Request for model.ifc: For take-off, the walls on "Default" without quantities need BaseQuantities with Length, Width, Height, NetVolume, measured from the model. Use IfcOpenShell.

First a look at what the model holds.

```python
import ifcopenshell
import ifcopenshell.util.element
import ifcopenshell.util.unit

model = ifcopenshell.open("model.ifc")
print(model.schema)
for unit_type in ("LENGTHUNIT", "AREAUNIT", "VOLUMEUNIT"):
    print(unit_type, ifcopenshell.util.unit.calculate_unit_scale(model, unit_type))
storey = next(s for s in model.by_type("IfcBuildingStorey") if s.Name == "Default")
walls = [e for e in ifcopenshell.util.element.get_decomposition(storey) if e.is_a("IfcWall")]
for e in sorted(walls, key=lambda e: e.id()):
    print(e.id(), e.is_a(), e.Name, list(ifcopenshell.util.element.get_psets(e, qtos_only=True)), sep=" | ")
```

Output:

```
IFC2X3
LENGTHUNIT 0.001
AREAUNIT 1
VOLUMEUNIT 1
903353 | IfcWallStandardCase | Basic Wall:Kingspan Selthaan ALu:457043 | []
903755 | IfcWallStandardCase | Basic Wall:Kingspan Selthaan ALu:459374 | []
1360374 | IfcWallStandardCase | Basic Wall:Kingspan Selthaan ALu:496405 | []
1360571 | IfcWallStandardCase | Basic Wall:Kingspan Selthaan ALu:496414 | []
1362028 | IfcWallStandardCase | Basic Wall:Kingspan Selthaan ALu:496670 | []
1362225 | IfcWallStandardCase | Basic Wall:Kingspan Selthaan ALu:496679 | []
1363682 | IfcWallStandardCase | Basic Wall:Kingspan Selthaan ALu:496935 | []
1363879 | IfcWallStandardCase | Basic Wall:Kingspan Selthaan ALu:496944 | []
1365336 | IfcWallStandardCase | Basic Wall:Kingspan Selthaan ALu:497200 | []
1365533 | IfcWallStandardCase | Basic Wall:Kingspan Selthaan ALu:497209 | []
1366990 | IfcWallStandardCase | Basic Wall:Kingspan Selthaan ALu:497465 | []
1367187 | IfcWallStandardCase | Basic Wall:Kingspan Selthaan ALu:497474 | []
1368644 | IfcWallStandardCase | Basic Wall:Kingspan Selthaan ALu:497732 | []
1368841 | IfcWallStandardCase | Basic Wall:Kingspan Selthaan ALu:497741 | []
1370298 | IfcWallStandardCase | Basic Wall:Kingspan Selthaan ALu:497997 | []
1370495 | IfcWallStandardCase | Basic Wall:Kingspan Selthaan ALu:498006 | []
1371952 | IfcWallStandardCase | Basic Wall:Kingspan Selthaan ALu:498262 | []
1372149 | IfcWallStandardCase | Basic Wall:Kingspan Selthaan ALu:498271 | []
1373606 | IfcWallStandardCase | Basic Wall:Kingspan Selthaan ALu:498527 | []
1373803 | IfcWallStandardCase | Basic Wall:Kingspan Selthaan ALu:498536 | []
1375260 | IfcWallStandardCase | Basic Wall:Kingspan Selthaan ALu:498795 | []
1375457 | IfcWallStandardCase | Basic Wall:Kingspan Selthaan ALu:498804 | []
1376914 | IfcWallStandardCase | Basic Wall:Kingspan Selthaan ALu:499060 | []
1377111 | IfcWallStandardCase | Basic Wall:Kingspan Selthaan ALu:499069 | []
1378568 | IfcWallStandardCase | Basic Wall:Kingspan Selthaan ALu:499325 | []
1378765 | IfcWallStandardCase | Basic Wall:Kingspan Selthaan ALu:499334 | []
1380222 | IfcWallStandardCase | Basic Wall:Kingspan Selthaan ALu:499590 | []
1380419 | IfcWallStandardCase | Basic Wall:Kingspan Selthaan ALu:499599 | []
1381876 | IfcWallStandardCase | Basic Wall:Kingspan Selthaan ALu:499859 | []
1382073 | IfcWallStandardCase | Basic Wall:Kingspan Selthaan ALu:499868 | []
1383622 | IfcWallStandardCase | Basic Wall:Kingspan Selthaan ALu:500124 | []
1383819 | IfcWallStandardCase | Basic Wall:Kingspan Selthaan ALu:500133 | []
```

```python
import ifcopenshell
import ifcopenshell.api.pset
import ifcopenshell.geom
import ifcopenshell.util.element
import ifcopenshell.util.shape
import ifcopenshell.util.unit

model = ifcopenshell.open("model.ifc")
unit_scale = ifcopenshell.util.unit.calculate_unit_scale(model)
volume_scale = ifcopenshell.util.unit.calculate_unit_scale(model, "VOLUMEUNIT")
settings = ifcopenshell.geom.settings()

storey = next(s for s in model.by_type("IfcBuildingStorey") if s.Name == "Default")
walls = [e for e in ifcopenshell.util.element.get_decomposition(storey) if e.is_a("IfcWall")]

for e in sorted(walls, key=lambda e: e.id()):
    if ifcopenshell.util.element.get_psets(e, qtos_only=True, should_inherit=False):
        continue
    # Geometry comes back in metres, in the element's own axes.
    shape = ifcopenshell.geom.create_shape(settings, e)
    values = {
        "Length": ifcopenshell.util.shape.get_x(shape.geometry) / unit_scale,
        "Width": ifcopenshell.util.shape.get_y(shape.geometry) / unit_scale,
        "Height": ifcopenshell.util.shape.get_z(shape.geometry) / unit_scale,
        "NetVolume": ifcopenshell.util.shape.get_volume(shape.geometry) / volume_scale,
    }
    qto = ifcopenshell.api.pset.add_qto(model, product=e, name="BaseQuantities")
    ifcopenshell.api.pset.edit_qto(model, qto=qto, properties=values)
    print(e.id(), {k: round(v, 3) for k, v in values.items()})

model.write("model_v2.ifc")
```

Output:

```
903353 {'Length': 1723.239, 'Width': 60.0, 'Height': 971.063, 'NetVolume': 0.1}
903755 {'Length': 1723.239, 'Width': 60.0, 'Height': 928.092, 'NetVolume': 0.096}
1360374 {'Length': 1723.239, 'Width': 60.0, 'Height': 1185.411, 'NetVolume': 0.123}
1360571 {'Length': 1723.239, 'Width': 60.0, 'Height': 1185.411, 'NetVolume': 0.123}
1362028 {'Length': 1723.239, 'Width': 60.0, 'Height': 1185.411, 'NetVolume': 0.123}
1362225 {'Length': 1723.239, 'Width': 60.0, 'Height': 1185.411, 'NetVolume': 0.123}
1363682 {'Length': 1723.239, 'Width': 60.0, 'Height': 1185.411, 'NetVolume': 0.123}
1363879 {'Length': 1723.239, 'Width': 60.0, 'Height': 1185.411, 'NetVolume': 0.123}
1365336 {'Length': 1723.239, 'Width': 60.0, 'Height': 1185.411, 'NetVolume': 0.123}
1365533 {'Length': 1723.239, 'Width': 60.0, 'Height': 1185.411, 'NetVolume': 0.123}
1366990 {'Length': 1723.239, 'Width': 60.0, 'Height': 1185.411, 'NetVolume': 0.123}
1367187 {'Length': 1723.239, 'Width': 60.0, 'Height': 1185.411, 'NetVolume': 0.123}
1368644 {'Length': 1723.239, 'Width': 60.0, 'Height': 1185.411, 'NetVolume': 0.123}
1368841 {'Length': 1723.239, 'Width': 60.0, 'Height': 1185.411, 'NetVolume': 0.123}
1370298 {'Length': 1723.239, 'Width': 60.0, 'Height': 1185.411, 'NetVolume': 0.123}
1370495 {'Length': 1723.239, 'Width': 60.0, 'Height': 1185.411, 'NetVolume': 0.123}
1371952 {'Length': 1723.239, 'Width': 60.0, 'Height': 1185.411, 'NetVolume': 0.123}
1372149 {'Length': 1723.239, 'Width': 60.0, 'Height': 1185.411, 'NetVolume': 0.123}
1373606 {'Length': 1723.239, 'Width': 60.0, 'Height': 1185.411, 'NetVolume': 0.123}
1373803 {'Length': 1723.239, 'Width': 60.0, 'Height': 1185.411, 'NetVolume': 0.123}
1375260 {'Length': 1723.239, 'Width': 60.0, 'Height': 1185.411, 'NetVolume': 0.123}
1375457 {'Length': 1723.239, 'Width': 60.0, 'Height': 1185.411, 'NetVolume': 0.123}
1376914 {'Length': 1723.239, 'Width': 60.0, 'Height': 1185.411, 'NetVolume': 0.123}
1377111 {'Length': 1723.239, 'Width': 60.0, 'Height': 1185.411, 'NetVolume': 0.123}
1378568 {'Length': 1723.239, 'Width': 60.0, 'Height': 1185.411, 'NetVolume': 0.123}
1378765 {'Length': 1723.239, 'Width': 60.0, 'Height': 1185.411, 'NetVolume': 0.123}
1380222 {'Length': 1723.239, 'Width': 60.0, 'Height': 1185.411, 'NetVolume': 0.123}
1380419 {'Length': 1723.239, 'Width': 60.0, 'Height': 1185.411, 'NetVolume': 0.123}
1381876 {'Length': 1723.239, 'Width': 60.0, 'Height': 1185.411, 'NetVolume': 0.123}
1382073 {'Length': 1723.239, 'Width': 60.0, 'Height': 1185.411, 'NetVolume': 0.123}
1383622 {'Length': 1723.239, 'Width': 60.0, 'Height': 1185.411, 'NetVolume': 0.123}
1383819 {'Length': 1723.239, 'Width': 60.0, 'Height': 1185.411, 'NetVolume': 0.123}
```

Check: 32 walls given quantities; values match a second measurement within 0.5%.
